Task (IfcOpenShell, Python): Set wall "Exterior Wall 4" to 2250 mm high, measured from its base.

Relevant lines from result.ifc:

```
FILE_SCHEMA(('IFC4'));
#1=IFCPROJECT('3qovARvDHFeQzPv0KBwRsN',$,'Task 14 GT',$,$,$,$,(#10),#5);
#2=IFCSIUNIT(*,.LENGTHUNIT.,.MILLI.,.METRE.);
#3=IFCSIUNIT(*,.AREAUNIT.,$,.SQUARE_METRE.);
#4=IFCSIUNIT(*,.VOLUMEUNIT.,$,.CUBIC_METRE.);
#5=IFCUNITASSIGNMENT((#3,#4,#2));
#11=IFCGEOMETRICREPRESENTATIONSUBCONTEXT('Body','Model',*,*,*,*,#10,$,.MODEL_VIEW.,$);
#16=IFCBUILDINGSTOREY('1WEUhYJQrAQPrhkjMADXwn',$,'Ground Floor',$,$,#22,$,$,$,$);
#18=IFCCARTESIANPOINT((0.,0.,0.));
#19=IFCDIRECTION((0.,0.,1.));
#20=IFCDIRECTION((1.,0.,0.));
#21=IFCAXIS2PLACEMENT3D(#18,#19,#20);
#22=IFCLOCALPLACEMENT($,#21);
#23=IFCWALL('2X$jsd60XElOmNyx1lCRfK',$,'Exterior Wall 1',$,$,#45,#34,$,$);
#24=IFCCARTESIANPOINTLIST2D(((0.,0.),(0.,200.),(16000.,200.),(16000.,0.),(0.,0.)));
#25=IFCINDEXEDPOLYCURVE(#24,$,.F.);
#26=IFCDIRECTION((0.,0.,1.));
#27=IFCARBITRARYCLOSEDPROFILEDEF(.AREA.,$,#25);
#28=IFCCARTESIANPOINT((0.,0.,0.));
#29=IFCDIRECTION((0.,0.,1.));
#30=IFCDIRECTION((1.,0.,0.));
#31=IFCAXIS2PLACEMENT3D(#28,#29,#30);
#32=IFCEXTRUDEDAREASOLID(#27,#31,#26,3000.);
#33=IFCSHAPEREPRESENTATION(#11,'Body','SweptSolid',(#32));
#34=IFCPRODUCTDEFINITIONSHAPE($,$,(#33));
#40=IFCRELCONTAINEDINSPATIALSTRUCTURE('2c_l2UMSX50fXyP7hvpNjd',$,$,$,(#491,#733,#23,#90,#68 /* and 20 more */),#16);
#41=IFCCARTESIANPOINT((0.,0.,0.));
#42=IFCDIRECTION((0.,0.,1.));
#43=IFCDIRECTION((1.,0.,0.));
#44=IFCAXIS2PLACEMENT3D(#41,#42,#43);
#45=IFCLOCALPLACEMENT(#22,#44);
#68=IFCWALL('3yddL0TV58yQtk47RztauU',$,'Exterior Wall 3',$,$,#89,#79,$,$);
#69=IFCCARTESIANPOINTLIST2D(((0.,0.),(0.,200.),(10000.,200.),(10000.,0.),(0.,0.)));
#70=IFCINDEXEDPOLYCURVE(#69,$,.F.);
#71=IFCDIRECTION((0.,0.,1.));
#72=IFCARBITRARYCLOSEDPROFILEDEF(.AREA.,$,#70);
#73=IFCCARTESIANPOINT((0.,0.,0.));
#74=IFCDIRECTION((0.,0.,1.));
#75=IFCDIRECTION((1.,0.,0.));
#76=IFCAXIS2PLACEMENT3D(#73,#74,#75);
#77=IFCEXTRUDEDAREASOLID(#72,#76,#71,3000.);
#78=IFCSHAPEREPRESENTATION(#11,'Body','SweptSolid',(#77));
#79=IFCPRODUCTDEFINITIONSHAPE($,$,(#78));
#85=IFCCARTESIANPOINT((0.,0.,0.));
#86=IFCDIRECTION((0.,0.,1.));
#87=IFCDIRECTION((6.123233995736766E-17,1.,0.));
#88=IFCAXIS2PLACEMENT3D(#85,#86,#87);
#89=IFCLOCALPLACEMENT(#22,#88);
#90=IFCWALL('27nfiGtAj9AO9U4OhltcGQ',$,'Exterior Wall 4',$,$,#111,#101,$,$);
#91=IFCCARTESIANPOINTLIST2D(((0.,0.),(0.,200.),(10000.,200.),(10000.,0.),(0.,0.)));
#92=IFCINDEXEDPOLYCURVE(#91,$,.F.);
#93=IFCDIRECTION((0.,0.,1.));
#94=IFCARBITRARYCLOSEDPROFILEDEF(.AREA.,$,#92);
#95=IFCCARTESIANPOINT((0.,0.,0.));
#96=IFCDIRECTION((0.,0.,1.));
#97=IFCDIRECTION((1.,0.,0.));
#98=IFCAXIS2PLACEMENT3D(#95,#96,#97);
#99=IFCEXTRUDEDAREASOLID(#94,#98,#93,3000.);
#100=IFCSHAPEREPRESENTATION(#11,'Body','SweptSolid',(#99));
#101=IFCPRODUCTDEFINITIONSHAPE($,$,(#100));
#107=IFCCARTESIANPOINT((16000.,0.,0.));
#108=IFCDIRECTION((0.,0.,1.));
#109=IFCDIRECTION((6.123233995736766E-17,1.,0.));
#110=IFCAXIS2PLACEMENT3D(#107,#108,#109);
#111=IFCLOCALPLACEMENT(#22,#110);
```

```python
import ifcopenshell
import ifcopenshell.geom
import ifcopenshell.util.representation
import ifcopenshell.util.shape
import ifcopenshell.util.unit

model = ifcopenshell.open("result.ifc")
unit_scale = ifcopenshell.util.unit.calculate_unit_scale(model)
settings = ifcopenshell.geom.settings()


def volume(element):
    """Net volume in cubic metres, openings subtracted."""
    shape = ifcopenshell.geom.create_shape(settings, element)
    return ifcopenshell.util.shape.get_volume(shape.geometry)


wall = model.by_guid("27nfiGtAj9AO9U4OhltcGQ")
before = volume(wall)

body = ifcopenshell.util.representation.get_representation(wall, "Model", "Body")
solid = body.Items[0]
old_height = solid.Depth
solid.Depth = 2.25 / unit_scale
after = volume(wall)

print(f"height {old_height:g} -> {solid.Depth:g}, volume {before:.3f} -> {after:.3f} m3")

model.write("result_v2.ifc")
```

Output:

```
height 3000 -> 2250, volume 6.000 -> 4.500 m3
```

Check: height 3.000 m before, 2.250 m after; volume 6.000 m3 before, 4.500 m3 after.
